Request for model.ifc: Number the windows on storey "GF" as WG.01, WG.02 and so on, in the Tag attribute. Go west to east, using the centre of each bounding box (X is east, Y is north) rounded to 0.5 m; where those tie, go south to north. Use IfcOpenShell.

First a look at what the model holds.

```python
import ifcopenshell
import ifcopenshell.util.element
import ifcopenshell.util.placement

model = ifcopenshell.open("model.ifc")
print(model.schema)
storey = next(s for s in model.by_type("IfcBuildingStorey") if s.Name == "GF")
windows = [e for e in ifcopenshell.util.element.get_decomposition(storey) if e.is_a("IfcWindow")]
for e in sorted(windows, key=lambda e: e.id()):
    origin = ifcopenshell.util.placement.get_local_placement(e.ObjectPlacement)[:3, 3]
    print(e.id(), e.Tag, e.Name, origin.round(2) + 0.0, sep=" | ")
```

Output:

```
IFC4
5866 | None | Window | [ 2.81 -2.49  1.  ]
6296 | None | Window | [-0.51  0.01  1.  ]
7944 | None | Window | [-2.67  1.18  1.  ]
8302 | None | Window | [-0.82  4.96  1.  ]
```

```python
import ifcopenshell
import ifcopenshell.geom
import ifcopenshell.util.element
import ifcopenshell.util.shape

model = ifcopenshell.open("model.ifc")
settings = ifcopenshell.geom.settings()
settings.set("use-world-coords", True)


def centre(element):
    shape = ifcopenshell.geom.create_shape(settings, element)
    return ifcopenshell.util.shape.get_bbox_centroid(shape.geometry)


storey = next(s for s in model.by_type("IfcBuildingStorey") if s.Name == "GF")
windows = [e for e in ifcopenshell.util.element.get_decomposition(storey) if e.is_a("IfcWindow")]

# Insertion points can sit at a corner or the storey origin, so sort by the geometry (in metres).
centres = {e: centre(e) for e in windows}
windows.sort(key=lambda e: (round(centres[e][0] / 0.5), centres[e][1]))

for i, e in enumerate(windows, start=1):
    number = f"WG.{i:02d}"
    e.Tag = number
    print(e.id(), number)

model.write("model_rev.ifc")
```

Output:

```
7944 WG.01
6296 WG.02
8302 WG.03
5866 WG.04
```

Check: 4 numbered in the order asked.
